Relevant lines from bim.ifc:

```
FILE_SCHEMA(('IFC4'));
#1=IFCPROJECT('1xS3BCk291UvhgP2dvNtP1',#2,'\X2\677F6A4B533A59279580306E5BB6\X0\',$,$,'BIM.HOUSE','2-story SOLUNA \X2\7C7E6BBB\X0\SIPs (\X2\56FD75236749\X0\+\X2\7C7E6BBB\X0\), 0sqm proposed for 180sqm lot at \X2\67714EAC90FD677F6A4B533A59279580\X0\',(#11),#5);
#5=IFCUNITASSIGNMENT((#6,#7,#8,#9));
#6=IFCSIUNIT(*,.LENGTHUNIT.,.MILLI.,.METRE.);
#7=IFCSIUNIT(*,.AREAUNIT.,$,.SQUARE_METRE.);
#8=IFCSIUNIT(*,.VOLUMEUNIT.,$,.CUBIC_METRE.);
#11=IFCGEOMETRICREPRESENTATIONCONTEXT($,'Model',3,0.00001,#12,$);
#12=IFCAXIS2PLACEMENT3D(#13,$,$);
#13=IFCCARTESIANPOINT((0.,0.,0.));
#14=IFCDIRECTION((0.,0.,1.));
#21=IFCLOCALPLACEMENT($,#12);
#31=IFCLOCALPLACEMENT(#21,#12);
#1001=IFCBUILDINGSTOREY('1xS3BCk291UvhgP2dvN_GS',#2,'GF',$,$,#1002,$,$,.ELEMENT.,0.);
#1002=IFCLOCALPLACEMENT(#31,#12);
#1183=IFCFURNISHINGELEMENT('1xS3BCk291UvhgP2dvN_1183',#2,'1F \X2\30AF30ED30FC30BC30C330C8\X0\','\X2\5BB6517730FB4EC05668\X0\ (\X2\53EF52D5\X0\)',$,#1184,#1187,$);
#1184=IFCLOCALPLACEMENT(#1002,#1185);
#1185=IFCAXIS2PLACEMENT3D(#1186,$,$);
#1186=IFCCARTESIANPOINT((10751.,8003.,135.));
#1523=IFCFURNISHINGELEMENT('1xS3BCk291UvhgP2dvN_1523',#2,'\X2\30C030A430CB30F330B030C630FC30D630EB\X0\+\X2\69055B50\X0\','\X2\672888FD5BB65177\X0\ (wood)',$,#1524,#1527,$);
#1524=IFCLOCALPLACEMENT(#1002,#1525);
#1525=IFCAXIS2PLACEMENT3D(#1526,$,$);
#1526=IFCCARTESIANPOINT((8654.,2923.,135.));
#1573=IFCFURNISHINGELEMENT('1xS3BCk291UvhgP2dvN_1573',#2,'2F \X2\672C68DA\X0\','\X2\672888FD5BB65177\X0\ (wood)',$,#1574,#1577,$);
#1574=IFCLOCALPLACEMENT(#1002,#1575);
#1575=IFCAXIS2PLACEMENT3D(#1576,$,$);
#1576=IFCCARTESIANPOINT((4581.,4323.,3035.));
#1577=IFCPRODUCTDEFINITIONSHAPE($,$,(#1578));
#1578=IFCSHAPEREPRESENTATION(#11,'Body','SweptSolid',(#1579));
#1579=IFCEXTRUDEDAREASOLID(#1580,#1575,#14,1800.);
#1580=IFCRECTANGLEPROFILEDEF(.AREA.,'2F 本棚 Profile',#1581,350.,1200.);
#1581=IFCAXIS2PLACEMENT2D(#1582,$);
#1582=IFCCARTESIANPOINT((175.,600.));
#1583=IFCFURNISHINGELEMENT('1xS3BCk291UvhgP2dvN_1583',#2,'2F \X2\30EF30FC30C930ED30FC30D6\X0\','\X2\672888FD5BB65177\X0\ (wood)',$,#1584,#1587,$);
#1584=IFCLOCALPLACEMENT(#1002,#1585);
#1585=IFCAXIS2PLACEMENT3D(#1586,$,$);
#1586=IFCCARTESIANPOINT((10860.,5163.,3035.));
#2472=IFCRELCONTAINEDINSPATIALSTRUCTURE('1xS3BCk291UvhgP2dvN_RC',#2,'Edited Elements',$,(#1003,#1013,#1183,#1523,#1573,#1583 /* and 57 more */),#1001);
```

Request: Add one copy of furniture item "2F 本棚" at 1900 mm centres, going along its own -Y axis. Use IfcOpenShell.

```python
import ifcopenshell
import ifcopenshell.api.geometry
import ifcopenshell.api.root
import ifcopenshell.util.element
import ifcopenshell.util.placement
import ifcopenshell.util.unit

model = ifcopenshell.open("bim.ifc")
unit_scale = ifcopenshell.util.unit.calculate_unit_scale(model)


def reuse_history(source, copy):
    """copy_class also copies each property set's owner history, people and application; keep the originals."""
    for rel in copy.IsDefinedBy:
        if rel.is_a("IfcRelDefinesByProperties") and (history := rel.RelatingPropertyDefinition.OwnerHistory):
            rel.RelatingPropertyDefinition.OwnerHistory = source.OwnerHistory
            ifcopenshell.util.element.remove_deep2(model, history)


source = model.by_guid("1xS3BCk291UvhgP2dvN_1573")
base = ifcopenshell.util.placement.get_local_placement(source.ObjectPlacement)
step = -base[:3, 1] * 1.9 / unit_scale

for i in range(1, 2):
    copy = ifcopenshell.api.root.copy_class(model, product=source)
    copy.Representation = ifcopenshell.util.element.copy_deep(
        model, source.Representation, exclude=["IfcGeometricRepresentationContext", "IfcRepresentationMap"]
    )
    reuse_history(source, copy)
    matrix = base.copy()
    matrix[:3, 3] += i * step
    print("added at", matrix[:3, 3].round(3) + 0.0)
    ifcopenshell.api.geometry.edit_object_placement(model, product=copy, matrix=matrix, is_si=False)

model.write("bim_rev.ifc")
```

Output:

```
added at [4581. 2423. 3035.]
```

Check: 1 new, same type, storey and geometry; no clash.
